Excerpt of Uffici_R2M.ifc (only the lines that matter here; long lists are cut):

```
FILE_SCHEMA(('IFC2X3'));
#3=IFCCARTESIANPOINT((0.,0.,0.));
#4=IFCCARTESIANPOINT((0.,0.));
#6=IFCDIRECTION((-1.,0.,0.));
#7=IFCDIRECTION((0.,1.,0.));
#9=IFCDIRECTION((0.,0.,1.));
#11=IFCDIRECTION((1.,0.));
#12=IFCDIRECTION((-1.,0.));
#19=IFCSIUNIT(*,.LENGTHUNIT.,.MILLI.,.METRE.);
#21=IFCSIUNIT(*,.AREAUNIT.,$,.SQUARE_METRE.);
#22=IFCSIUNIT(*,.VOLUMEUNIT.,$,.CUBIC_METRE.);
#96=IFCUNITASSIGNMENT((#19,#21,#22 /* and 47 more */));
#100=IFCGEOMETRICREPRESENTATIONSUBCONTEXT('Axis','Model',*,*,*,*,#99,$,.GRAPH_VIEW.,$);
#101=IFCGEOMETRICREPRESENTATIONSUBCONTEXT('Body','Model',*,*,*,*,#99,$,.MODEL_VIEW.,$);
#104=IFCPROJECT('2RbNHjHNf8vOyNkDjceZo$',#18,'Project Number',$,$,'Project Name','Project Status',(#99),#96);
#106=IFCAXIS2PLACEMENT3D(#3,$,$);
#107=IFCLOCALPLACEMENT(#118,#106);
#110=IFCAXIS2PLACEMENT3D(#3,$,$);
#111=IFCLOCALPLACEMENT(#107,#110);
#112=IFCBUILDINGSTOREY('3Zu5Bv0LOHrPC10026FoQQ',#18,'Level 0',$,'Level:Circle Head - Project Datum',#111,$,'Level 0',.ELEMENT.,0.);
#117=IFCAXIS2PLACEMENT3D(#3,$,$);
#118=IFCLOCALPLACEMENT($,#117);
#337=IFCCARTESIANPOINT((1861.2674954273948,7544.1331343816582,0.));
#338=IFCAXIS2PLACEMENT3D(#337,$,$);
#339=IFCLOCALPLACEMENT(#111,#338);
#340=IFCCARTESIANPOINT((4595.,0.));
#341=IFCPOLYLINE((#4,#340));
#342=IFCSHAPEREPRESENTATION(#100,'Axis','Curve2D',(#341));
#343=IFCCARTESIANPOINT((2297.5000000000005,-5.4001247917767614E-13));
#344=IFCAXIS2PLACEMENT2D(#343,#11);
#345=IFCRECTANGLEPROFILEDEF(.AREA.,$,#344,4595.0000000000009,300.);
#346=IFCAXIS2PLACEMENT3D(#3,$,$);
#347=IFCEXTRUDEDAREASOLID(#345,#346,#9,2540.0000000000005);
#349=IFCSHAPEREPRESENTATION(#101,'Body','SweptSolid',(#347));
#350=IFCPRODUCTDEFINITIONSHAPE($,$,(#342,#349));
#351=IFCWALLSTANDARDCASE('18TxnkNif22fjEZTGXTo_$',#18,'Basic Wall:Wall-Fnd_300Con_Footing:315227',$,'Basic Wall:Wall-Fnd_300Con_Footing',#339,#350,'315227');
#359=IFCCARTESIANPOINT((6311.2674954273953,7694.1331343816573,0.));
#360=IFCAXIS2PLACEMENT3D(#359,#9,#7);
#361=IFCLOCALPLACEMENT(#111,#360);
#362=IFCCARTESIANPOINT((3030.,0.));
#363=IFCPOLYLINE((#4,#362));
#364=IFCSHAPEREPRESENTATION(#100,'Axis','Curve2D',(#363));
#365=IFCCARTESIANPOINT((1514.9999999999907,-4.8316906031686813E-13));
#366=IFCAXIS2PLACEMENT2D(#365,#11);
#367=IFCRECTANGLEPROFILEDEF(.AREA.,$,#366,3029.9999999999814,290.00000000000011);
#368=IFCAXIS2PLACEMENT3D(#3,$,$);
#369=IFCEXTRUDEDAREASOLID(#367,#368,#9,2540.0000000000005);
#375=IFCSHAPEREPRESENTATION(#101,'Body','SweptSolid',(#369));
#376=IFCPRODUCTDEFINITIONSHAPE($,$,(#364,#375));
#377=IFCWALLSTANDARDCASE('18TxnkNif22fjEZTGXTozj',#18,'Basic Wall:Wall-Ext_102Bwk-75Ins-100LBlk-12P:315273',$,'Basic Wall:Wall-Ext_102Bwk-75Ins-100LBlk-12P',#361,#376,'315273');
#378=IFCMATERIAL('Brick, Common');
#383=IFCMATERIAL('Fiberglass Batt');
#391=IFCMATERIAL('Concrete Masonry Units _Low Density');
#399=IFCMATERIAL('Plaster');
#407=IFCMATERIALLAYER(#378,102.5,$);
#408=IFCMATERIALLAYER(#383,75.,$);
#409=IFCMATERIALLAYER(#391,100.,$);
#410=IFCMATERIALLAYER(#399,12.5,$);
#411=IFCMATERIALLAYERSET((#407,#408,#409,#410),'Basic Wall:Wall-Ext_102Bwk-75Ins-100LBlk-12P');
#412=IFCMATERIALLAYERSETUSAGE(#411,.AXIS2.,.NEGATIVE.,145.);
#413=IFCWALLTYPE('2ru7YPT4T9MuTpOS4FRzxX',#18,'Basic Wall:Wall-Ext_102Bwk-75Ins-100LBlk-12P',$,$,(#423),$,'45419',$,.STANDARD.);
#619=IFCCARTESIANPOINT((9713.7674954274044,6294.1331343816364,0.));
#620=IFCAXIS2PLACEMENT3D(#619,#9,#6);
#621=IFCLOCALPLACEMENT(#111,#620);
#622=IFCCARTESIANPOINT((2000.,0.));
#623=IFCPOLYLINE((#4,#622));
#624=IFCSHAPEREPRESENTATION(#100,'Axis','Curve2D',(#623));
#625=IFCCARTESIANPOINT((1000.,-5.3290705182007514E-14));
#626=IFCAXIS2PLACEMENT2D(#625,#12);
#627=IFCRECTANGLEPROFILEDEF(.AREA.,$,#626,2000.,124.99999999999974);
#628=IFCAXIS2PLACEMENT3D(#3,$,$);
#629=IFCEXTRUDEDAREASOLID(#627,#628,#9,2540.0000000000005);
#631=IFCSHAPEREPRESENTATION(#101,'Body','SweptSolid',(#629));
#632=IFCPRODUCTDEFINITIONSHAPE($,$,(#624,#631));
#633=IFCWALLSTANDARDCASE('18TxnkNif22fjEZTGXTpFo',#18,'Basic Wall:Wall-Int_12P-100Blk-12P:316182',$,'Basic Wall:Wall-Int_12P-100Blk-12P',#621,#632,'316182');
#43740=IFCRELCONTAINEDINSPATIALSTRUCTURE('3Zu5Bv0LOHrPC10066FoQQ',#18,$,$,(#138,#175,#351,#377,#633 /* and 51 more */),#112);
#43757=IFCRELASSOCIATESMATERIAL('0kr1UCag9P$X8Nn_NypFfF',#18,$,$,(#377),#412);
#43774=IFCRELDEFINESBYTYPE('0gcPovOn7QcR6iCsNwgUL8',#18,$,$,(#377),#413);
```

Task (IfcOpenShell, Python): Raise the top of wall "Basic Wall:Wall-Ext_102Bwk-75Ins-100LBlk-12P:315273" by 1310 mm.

```python
import ifcopenshell
import ifcopenshell.geom
import ifcopenshell.util.representation
import ifcopenshell.util.shape
import ifcopenshell.util.unit

model = ifcopenshell.open("Uffici_R2M.ifc")
unit_scale = ifcopenshell.util.unit.calculate_unit_scale(model)
settings = ifcopenshell.geom.settings()


def volume(element):
    """Net volume in cubic metres, openings subtracted."""
    shape = ifcopenshell.geom.create_shape(settings, element)
    return ifcopenshell.util.shape.get_volume(shape.geometry)


wall = model.by_id(377)
before = volume(wall)

body = ifcopenshell.util.representation.get_representation(wall, "Model", "Body")
solid = body.Items[0]
old_height = solid.Depth
solid.Depth += 1.31 / unit_scale
after = volume(wall)

print(f"height {old_height:g} -> {solid.Depth:g}, volume {before:.3f} -> {after:.3f} m3")

model.write("Uffici_R2M-out.ifc")
```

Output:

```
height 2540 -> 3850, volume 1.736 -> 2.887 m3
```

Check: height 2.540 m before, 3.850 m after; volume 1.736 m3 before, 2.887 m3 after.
